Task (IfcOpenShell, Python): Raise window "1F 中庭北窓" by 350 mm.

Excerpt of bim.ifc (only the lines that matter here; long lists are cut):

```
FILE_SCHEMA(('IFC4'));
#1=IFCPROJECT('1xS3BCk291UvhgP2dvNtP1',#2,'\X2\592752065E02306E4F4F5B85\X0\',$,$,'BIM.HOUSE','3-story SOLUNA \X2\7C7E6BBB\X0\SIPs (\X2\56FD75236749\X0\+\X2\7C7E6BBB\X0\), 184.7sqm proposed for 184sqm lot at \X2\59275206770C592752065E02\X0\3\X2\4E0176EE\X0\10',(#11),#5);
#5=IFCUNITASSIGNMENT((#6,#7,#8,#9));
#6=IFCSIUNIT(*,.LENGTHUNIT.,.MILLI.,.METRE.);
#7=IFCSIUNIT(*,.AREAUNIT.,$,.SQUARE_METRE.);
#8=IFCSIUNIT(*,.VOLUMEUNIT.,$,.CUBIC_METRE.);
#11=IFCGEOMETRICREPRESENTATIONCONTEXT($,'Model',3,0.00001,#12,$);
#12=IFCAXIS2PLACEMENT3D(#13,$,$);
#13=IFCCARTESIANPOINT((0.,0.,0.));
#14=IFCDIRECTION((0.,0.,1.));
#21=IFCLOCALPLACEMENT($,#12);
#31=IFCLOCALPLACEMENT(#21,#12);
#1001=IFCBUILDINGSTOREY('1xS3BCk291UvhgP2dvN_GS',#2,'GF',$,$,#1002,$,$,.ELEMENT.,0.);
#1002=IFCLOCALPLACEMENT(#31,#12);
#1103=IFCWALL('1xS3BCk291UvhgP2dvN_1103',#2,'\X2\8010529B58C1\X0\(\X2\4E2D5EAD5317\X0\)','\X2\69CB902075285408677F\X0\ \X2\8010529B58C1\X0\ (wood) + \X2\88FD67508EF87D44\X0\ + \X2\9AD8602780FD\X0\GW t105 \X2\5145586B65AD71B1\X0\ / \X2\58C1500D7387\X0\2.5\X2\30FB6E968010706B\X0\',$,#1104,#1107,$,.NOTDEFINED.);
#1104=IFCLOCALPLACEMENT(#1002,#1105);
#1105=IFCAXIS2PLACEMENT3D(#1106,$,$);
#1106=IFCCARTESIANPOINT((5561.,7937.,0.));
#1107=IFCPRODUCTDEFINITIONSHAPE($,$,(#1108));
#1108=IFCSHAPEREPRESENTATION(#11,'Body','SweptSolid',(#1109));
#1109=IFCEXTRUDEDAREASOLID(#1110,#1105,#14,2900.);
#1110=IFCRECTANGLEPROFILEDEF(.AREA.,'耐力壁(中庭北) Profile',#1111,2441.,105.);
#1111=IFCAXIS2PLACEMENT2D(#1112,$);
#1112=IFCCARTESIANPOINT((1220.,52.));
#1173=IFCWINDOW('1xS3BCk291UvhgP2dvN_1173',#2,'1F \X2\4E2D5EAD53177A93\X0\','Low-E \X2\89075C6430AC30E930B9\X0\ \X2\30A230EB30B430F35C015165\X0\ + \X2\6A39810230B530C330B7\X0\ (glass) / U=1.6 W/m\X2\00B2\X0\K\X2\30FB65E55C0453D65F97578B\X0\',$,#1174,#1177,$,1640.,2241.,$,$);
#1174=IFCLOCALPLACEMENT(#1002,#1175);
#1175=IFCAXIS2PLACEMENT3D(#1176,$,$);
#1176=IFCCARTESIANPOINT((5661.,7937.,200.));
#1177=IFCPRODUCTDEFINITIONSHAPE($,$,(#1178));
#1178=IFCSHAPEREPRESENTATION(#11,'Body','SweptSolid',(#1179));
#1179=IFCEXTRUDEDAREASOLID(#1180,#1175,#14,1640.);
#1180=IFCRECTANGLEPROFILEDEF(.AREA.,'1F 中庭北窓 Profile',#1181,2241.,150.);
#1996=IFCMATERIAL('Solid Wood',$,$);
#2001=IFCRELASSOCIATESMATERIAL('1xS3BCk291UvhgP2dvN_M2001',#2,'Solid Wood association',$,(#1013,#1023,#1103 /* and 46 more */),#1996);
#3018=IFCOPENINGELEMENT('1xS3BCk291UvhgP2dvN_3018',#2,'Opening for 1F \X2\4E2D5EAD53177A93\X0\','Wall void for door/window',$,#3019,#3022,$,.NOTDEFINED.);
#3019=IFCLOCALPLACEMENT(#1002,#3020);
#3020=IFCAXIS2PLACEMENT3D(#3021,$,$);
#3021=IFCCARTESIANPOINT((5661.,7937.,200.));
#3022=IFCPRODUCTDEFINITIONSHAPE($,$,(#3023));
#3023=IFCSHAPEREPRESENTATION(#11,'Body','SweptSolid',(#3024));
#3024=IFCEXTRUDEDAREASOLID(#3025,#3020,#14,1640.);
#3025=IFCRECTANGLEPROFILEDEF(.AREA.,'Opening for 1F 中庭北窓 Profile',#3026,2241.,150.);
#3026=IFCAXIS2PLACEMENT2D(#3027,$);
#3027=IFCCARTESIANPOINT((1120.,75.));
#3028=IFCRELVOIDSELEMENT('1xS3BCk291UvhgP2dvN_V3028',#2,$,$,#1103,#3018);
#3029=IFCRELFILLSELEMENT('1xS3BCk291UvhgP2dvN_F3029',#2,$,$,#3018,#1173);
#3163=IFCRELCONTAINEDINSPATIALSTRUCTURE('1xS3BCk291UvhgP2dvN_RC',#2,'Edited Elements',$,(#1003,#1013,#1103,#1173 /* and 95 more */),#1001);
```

```python
import numpy as np
import ifcopenshell
import ifcopenshell.api.geometry
import ifcopenshell.util.placement
import ifcopenshell.util.unit

model = ifcopenshell.open("bim.ifc")
unit_scale = ifcopenshell.util.unit.calculate_unit_scale(model)

window = model.by_guid("1xS3BCk291UvhgP2dvN_1173")
opening = window.FillsVoids[0].RelatingOpeningElement
dz = 350.0

shift = np.array([0.0, 0.0, dz])
# The window is not placed relative to its opening, so move both.
for product in (opening, window):
    matrix = ifcopenshell.util.placement.get_local_placement(product.ObjectPlacement)
    matrix[:3, 3] += shift
    ifcopenshell.api.geometry.edit_object_placement(model, product=product, matrix=matrix, is_si=False)

print(f"moved by {dz * unit_scale:+.3f} m")

model.write("bim-out.ifc")
```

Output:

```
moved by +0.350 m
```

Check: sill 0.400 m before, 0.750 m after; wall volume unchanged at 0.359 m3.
